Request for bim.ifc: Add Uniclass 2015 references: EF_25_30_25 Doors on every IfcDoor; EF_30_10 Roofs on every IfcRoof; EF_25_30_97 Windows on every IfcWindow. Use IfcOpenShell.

First a look at what the model holds.

```python
import ifcopenshell

model = ifcopenshell.open("bim.ifc")
print(model.schema)
print("classifications:", [c.Name for c in model.by_type("IfcClassification")])
for ifc_class in ("IfcDoor", "IfcRoof", "IfcStair", "IfcWall", "IfcWindow"):
    print(ifc_class, len(model.by_type(ifc_class)))
```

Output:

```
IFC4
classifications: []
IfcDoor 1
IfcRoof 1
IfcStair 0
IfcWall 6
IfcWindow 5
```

```python
import ifcopenshell
import ifcopenshell.api.classification

model = ifcopenshell.open("bim.ifc")

system = ifcopenshell.api.classification.add_classification(model, classification="Uniclass 2015")

codes = {
    "IfcDoor": ("EF_25_30_25", "Doors"),
    "IfcRoof": ("EF_30_10", "Roofs"),
    "IfcWindow": ("EF_25_30_97", "Windows"),
}
for ifc_class, (code, name) in codes.items():
    products = model.by_type(ifc_class)
    ifcopenshell.api.classification.add_reference(
        model, products=products, classification=system, identification=code, name=name
    )
    print(code, len(products))

model.write("bim_edited.ifc")
```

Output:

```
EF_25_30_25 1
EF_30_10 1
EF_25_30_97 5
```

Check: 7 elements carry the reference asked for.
